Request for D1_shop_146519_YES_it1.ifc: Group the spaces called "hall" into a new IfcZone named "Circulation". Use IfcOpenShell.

First a look at what the model holds.

```python
import ifcopenshell

model = ifcopenshell.open("D1_shop_146519_YES_it1.ifc")
print(model.schema)
seen = {}
for space in model.by_type("IfcSpace"):
    seen[space.LongName] = seen.get(space.LongName, 0) + 1
for name, count in sorted(seen.items(), key=str):
    print(count, "x", name)
print("zones:", [z.Name for z in model.by_type("IfcZone")][:20])
```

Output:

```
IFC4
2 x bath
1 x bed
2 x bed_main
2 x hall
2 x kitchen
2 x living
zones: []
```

```python
import ifcopenshell
import ifcopenshell.api.group
import ifcopenshell.api.root

model = ifcopenshell.open("D1_shop_146519_YES_it1.ifc")

names = {"hall"}
spaces = [s for s in model.by_type("IfcSpace") if s.LongName in names]

zone = ifcopenshell.api.root.create_entity(model, ifc_class="IfcZone", name="Circulation")
ifcopenshell.api.group.assign_group(model, products=spaces, group=zone)
print(len(spaces), "spaces in", zone.Name)

model.write("D1_shop_146519_YES_it1_edited.ifc")
```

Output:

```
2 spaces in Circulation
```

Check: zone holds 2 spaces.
